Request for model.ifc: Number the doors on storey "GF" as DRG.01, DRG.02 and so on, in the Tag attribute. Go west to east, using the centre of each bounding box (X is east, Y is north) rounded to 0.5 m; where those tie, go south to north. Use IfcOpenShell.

First a look at what the model holds.

```python
import ifcopenshell
import ifcopenshell.util.element
import ifcopenshell.util.placement

model = ifcopenshell.open("model.ifc")
print(model.schema)
storey = next(s for s in model.by_type("IfcBuildingStorey") if s.Name == "GF")
doors = [e for e in ifcopenshell.util.element.get_decomposition(storey) if e.is_a("IfcDoor")]
for e in sorted(doors, key=lambda e: e.id()):
    origin = ifcopenshell.util.placement.get_local_placement(e.ObjectPlacement)[:3, 3]
    print(e.id(), e.Tag, e.Name, origin.round(2) + 0.0, sep=" | ")
```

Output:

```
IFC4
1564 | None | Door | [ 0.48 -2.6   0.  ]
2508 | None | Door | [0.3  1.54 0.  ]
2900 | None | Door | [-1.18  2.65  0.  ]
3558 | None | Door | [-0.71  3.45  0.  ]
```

```python
import ifcopenshell
import ifcopenshell.geom
import ifcopenshell.util.element
import ifcopenshell.util.shape

model = ifcopenshell.open("model.ifc")
settings = ifcopenshell.geom.settings()
settings.set("use-world-coords", True)


def centre(element):
    shape = ifcopenshell.geom.create_shape(settings, element)
    return ifcopenshell.util.shape.get_bbox_centroid(shape.geometry)


storey = next(s for s in model.by_type("IfcBuildingStorey") if s.Name == "GF")
doors = [e for e in ifcopenshell.util.element.get_decomposition(storey) if e.is_a("IfcDoor")]

# Insertion points can sit at a corner or the storey origin, so sort by the geometry (in metres).
centres = {e: centre(e) for e in doors}
doors.sort(key=lambda e: (round(centres[e][0] / 0.5), centres[e][1]))

for i, e in enumerate(doors, start=1):
    number = f"DRG.{i:02d}"
    e.Tag = number
    print(e.id(), number)

model.write("model_updated.ifc")
```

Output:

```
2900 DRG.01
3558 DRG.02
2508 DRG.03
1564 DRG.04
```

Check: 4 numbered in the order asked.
